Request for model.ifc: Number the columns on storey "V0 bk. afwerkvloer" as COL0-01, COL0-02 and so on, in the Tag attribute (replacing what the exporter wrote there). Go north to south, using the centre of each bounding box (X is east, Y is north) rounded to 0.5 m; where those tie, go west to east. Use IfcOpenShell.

First a look at what the model holds.

```python
import ifcopenshell
import ifcopenshell.util.element
import ifcopenshell.util.placement

model = ifcopenshell.open("model.ifc")
print(model.schema)
storey = next(s for s in model.by_type("IfcBuildingStorey") if s.Name == "V0 bk. afwerkvloer")
columns = [e for e in ifcopenshell.util.element.get_decomposition(storey) if e.is_a("IfcColumn")]
for e in sorted(columns, key=lambda e: e.id()):
    origin = ifcopenshell.util.placement.get_local_placement(e.ObjectPlacement)[:3, 3]
    print(e.id(), e.Tag, e.Name, origin.round(2) + 0.0, sep=" | ")
```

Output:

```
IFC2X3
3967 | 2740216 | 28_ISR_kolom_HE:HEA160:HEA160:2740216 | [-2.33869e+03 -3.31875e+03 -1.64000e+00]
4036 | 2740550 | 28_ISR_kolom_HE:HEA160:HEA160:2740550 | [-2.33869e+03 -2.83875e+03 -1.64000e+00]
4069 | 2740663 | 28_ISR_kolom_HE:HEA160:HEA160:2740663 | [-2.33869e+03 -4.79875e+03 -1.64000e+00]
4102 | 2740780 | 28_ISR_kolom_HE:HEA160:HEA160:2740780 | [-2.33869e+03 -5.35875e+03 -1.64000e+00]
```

```python
import ifcopenshell
import ifcopenshell.geom
import ifcopenshell.util.element
import ifcopenshell.util.shape

model = ifcopenshell.open("model.ifc")
settings = ifcopenshell.geom.settings()
settings.set("use-world-coords", True)


def centre(element):
    shape = ifcopenshell.geom.create_shape(settings, element)
    return ifcopenshell.util.shape.get_bbox_centroid(shape.geometry)


storey = next(s for s in model.by_type("IfcBuildingStorey") if s.Name == "V0 bk. afwerkvloer")
columns = [e for e in ifcopenshell.util.element.get_decomposition(storey) if e.is_a("IfcColumn")]

# Insertion points can sit at a corner or the storey origin, so sort by the geometry (in metres).
centres = {e: centre(e) for e in columns}
columns.sort(key=lambda e: (-round(centres[e][1] / 0.5), centres[e][0]))

for i, e in enumerate(columns, start=1):
    number = f"COL0-{i:02d}"
    e.Tag = number
    print(e.id(), number)

model.write("model_rev.ifc")
```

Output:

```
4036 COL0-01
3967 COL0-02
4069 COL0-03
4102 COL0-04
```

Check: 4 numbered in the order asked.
